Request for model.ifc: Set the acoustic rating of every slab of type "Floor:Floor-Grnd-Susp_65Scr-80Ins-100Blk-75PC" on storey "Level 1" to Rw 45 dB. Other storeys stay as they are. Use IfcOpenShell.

First a look at what the model holds.

```python
import ifcopenshell
import ifcopenshell.util.element

model = ifcopenshell.open("model.ifc")
print(model.schema)
storey = next(s for s in model.by_type("IfcBuildingStorey") if s.Name == "Level 1")
slabs = [e for e in ifcopenshell.util.element.get_decomposition(storey) if e.is_a("IfcSlab")]
seen = {}
for e in slabs:
    element_type = ifcopenshell.util.element.get_type(e)
    key = (element_type.Name if element_type != e and element_type else None, ifcopenshell.util.element.get_pset(e, "Pset_SlabCommon", "AcousticRating"))
    seen[key] = seen.get(key, 0) + 1
for (name, value), count in sorted(seen.items(), key=str):
    print(count, "x", name, "|", value)
```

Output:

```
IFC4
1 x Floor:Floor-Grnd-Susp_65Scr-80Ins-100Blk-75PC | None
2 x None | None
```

```python
import ifcopenshell
import ifcopenshell.api.pset
import ifcopenshell.util.element

model = ifcopenshell.open("model.ifc")

storey = next(s for s in model.by_type("IfcBuildingStorey") if s.Name == "Level 1")
slabs = [e for e in ifcopenshell.util.element.get_decomposition(storey) if e.is_a("IfcSlab")]

count = 0
for e in slabs:
    element_type = ifcopenshell.util.element.get_type(e)
    if element_type in (None, e) or element_type.Name != "Floor:Floor-Grnd-Susp_65Scr-80Ins-100Blk-75PC":
        continue
    # add_pset returns the element's existing set when there is one.
    pset = ifcopenshell.api.pset.add_pset(model, product=e, name="Pset_SlabCommon")
    ifcopenshell.api.pset.edit_pset(model, pset=pset, properties={"AcousticRating": "Rw 45 dB"})
    count += 1

print(count, "slabs updated")

model.write("model_rev.ifc")
```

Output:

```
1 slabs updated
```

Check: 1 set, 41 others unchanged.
